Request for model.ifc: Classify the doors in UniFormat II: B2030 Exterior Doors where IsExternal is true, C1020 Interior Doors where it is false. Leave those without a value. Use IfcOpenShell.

First a look at what the model holds.

```python
import ifcopenshell
import ifcopenshell.util.element

model = ifcopenshell.open("model.ifc")
print(model.schema)
print("classifications:", [c.Name for c in model.by_type("IfcClassification")])
values = [ifcopenshell.util.element.get_pset(e, "Pset_DoorCommon", "IsExternal") for e in model.by_type("IfcDoor")]
for value in (True, False, None):
    print("IsExternal", value, values.count(value))
```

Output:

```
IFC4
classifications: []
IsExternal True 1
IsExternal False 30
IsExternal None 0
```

```python
import ifcopenshell
import ifcopenshell.api.classification
import ifcopenshell.util.element

model = ifcopenshell.open("model.ifc")

system = ifcopenshell.api.classification.add_classification(model, classification="UniFormat II")

doors = model.by_type("IfcDoor")
external = {e: ifcopenshell.util.element.get_pset(e, "Pset_DoorCommon", "IsExternal") for e in doors}
for flag, code, name in ((True, "B2030", "Exterior Doors"), (False, "C1020", "Interior Doors")):
    products = [e for e in doors if external[e] is flag]
    ifcopenshell.api.classification.add_reference(
        model, products=products, classification=system, identification=code, name=name
    )
    print(code, len(products))

model.write("model_v2.ifc")
```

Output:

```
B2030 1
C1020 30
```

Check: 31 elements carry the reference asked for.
